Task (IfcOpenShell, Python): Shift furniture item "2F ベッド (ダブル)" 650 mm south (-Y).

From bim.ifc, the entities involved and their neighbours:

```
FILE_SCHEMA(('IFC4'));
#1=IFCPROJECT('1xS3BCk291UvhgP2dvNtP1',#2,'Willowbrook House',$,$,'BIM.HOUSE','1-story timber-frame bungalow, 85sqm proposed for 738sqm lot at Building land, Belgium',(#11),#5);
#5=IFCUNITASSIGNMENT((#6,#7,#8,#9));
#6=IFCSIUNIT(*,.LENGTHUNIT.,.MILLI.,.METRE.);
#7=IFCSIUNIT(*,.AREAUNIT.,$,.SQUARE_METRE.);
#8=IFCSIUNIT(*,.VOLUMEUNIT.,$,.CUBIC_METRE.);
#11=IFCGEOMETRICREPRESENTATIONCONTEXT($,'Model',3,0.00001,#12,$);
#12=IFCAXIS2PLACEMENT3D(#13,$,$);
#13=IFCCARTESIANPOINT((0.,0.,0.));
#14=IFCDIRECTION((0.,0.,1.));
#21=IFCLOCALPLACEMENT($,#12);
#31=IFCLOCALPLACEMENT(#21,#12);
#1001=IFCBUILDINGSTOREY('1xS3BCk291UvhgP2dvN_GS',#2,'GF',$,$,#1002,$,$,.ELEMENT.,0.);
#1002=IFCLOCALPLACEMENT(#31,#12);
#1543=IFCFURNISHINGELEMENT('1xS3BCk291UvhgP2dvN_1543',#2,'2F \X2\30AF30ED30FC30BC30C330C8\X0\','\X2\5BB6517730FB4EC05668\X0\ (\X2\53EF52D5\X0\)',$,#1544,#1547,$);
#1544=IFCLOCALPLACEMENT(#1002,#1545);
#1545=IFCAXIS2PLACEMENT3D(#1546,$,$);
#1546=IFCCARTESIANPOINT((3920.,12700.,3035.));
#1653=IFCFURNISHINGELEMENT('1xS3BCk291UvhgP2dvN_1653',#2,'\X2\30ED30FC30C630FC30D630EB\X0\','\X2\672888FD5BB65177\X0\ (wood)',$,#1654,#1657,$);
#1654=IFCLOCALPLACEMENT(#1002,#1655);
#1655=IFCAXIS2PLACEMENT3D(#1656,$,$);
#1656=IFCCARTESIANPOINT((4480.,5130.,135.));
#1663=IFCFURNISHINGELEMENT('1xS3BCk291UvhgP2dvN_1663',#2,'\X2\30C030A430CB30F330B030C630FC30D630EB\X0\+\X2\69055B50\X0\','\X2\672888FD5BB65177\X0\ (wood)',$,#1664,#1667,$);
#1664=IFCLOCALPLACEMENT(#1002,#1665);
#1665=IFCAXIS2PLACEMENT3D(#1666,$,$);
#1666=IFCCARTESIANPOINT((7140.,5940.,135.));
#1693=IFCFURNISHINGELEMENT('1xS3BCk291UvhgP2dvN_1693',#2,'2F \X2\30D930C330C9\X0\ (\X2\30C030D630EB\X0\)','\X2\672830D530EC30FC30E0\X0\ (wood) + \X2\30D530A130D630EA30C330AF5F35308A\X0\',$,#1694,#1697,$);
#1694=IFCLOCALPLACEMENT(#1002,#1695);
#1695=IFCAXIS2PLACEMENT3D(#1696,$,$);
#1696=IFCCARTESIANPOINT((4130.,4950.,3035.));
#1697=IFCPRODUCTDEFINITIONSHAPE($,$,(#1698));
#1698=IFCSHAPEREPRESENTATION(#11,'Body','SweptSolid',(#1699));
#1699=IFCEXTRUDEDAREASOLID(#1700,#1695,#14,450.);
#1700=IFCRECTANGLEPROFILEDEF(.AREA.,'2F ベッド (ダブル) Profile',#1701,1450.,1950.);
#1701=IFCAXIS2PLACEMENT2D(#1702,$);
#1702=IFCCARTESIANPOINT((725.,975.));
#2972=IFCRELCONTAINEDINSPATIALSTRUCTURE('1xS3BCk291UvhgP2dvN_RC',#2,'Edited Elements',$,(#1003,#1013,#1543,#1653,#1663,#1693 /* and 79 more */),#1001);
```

```python
import ifcopenshell
import ifcopenshell.api.geometry
import ifcopenshell.util.placement

model = ifcopenshell.open("bim.ifc")

item = model.by_guid("1xS3BCk291UvhgP2dvN_1693")
matrix = ifcopenshell.util.placement.get_local_placement(item.ObjectPlacement)
matrix[1, 3] -= 650.0
ifcopenshell.api.geometry.edit_object_placement(model, product=item, matrix=matrix, is_si=False)

print(ifcopenshell.util.placement.get_local_placement(item.ObjectPlacement).round(3) + 0.0)

model.write("bim_edited.ifc")
```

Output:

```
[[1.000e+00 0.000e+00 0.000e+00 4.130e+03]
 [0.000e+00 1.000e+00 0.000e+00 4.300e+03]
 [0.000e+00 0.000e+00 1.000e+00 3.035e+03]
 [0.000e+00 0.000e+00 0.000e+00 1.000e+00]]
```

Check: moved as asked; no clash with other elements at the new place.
